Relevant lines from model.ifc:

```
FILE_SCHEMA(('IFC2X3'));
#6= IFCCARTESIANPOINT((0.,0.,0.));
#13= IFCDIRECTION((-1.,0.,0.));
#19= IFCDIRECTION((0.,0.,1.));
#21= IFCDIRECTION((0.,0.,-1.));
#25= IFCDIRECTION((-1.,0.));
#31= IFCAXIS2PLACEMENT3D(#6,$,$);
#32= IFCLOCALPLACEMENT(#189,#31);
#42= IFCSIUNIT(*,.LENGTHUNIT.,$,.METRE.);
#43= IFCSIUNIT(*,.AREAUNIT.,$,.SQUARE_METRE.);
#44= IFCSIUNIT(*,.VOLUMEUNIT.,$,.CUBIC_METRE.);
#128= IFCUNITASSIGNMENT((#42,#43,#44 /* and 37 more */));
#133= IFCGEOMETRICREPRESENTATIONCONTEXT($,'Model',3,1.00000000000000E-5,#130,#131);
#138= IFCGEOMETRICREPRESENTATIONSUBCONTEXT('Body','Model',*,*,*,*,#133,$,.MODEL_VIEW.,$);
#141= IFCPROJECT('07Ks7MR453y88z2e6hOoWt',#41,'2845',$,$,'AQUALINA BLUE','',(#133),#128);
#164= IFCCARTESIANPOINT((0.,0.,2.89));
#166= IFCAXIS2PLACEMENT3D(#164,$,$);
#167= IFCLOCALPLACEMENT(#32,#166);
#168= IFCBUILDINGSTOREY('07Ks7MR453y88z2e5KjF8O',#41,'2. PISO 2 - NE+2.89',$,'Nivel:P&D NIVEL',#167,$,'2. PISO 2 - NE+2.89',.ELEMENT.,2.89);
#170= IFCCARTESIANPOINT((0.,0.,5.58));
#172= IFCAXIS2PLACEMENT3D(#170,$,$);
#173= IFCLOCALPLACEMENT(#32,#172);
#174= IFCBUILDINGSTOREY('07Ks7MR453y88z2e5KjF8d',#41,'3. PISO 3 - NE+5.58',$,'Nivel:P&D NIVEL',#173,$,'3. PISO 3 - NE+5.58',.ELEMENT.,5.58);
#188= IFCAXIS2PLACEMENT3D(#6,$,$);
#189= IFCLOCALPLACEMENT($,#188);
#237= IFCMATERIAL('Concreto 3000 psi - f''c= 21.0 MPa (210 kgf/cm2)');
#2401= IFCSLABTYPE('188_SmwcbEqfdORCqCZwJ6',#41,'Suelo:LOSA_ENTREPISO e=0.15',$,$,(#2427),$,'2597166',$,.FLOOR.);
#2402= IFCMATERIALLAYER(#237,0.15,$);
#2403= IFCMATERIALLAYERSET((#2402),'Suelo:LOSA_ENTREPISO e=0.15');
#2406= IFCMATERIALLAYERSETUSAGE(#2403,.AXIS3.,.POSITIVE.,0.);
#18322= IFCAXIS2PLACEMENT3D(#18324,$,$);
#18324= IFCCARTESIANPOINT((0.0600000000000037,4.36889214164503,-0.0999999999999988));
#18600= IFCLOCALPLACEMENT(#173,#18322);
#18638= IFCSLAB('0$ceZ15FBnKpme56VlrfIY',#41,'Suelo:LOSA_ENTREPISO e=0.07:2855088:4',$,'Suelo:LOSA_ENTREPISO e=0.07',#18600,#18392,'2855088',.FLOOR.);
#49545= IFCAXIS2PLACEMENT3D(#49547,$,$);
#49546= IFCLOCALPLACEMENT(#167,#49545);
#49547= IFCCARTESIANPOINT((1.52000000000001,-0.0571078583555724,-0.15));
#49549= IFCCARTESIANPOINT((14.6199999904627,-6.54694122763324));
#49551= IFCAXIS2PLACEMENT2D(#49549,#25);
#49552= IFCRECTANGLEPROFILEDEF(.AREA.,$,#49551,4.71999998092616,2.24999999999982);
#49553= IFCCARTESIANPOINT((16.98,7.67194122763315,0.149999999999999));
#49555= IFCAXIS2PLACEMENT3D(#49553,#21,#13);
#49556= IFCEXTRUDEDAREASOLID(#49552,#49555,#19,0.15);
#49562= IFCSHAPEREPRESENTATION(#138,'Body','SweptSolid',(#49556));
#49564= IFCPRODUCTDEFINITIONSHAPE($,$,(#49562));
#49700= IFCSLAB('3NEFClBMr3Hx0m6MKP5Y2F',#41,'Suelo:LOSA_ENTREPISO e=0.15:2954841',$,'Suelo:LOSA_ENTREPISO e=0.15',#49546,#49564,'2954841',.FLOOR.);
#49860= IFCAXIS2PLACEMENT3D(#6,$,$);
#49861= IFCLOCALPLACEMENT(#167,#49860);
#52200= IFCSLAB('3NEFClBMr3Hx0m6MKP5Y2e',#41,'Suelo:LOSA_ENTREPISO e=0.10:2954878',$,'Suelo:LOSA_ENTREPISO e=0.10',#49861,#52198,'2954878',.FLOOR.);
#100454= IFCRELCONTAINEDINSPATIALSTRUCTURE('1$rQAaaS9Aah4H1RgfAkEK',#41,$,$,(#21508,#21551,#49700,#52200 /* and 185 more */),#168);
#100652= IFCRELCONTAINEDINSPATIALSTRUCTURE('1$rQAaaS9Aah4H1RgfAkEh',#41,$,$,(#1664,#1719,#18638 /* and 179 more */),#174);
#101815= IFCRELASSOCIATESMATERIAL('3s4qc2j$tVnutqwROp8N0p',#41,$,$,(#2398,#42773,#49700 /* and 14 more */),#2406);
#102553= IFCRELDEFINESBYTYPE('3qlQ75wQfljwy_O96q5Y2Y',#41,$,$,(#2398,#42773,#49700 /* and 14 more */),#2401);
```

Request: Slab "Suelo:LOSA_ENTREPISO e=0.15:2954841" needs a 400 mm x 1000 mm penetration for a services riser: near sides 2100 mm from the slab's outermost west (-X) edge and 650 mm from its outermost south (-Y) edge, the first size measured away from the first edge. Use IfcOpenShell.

```python
import numpy as np
import ifcopenshell
import ifcopenshell.api.feature
import ifcopenshell.api.geometry
import ifcopenshell.api.root
import ifcopenshell.geom
import ifcopenshell.util.placement
import ifcopenshell.util.representation
import ifcopenshell.util.shape
import ifcopenshell.util.unit

model = ifcopenshell.open("model.ifc")
unit_scale = ifcopenshell.util.unit.calculate_unit_scale(model)
settings = ifcopenshell.geom.settings()


def volume(element):
    """Net volume in cubic metres, openings subtracted."""
    shape = ifcopenshell.geom.create_shape(settings, element)
    return ifcopenshell.util.shape.get_volume(shape.geometry)


slab = model.by_guid("3NEFClBMr3Hx0m6MKP5Y2F")
before = volume(slab)

# Extent in the slab's own axes, in metres. The edges named are its -X and -Y sides.
slab_shape = ifcopenshell.geom.create_shape(settings, slab)
vertices = ifcopenshell.util.shape.get_vertices(slab_shape.geometry)
x_min, y_min, bottom = vertices.min(axis=0)
top = vertices[:, 2].max()

opening = ifcopenshell.api.root.create_entity(model, ifc_class="IfcOpeningElement", name="Services riser opening")
context = ifcopenshell.util.representation.get_context(model, "Model", "Body", "MODEL_VIEW")
width, depth = 0.4, 1
outline = [(0.0, 0.0), (width, 0.0), (width, depth), (0.0, depth), (0.0, 0.0)]
# Overshoot both faces by 50 mm so the cut is clean.
shape = ifcopenshell.api.geometry.add_slab_representation(
    model, context=context, depth=top - bottom + 0.1, polyline=outline
)
ifcopenshell.api.geometry.assign_representation(model, product=opening, representation=shape)

matrix = ifcopenshell.util.placement.get_local_placement(slab.ObjectPlacement)
matrix[:, 3] = matrix @ np.append(np.array([x_min + 2.1, y_min + 0.65, bottom - 0.05]) / unit_scale, 1.0)
ifcopenshell.api.geometry.edit_object_placement(model, product=opening, matrix=matrix, is_si=False)
ifcopenshell.api.feature.add_feature(model, feature=opening, element=slab)

after = volume(slab)

print(f"slab volume {before:.3f} -> {after:.3f} m3")

model.write("model_updated.ifc")
```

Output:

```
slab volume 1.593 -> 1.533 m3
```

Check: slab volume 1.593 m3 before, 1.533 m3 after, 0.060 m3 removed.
